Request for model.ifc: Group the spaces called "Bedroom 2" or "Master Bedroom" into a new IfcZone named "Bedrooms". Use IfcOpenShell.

First a look at what the model holds.

```python
import ifcopenshell

model = ifcopenshell.open("model.ifc")
print(model.schema)
seen = {}
for space in model.by_type("IfcSpace"):
    seen[space.LongName] = seen.get(space.LongName, 0) + 1
for name, count in sorted(seen.items(), key=str):
    print(count, "x", name)
print("zones:", [z.Name for z in model.by_type("IfcZone")][:20])
```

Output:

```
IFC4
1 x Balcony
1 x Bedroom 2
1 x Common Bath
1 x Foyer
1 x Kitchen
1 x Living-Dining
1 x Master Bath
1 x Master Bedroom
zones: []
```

```python
import ifcopenshell
import ifcopenshell.api.group
import ifcopenshell.api.root

model = ifcopenshell.open("model.ifc")

names = {"Bedroom 2", "Master Bedroom"}
spaces = [s for s in model.by_type("IfcSpace") if s.LongName in names]

zone = ifcopenshell.api.root.create_entity(model, ifc_class="IfcZone", name="Bedrooms")
ifcopenshell.api.group.assign_group(model, products=spaces, group=zone)
print(len(spaces), "spaces in", zone.Name)

model.write("model_rev.ifc")
```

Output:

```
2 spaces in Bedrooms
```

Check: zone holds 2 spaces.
